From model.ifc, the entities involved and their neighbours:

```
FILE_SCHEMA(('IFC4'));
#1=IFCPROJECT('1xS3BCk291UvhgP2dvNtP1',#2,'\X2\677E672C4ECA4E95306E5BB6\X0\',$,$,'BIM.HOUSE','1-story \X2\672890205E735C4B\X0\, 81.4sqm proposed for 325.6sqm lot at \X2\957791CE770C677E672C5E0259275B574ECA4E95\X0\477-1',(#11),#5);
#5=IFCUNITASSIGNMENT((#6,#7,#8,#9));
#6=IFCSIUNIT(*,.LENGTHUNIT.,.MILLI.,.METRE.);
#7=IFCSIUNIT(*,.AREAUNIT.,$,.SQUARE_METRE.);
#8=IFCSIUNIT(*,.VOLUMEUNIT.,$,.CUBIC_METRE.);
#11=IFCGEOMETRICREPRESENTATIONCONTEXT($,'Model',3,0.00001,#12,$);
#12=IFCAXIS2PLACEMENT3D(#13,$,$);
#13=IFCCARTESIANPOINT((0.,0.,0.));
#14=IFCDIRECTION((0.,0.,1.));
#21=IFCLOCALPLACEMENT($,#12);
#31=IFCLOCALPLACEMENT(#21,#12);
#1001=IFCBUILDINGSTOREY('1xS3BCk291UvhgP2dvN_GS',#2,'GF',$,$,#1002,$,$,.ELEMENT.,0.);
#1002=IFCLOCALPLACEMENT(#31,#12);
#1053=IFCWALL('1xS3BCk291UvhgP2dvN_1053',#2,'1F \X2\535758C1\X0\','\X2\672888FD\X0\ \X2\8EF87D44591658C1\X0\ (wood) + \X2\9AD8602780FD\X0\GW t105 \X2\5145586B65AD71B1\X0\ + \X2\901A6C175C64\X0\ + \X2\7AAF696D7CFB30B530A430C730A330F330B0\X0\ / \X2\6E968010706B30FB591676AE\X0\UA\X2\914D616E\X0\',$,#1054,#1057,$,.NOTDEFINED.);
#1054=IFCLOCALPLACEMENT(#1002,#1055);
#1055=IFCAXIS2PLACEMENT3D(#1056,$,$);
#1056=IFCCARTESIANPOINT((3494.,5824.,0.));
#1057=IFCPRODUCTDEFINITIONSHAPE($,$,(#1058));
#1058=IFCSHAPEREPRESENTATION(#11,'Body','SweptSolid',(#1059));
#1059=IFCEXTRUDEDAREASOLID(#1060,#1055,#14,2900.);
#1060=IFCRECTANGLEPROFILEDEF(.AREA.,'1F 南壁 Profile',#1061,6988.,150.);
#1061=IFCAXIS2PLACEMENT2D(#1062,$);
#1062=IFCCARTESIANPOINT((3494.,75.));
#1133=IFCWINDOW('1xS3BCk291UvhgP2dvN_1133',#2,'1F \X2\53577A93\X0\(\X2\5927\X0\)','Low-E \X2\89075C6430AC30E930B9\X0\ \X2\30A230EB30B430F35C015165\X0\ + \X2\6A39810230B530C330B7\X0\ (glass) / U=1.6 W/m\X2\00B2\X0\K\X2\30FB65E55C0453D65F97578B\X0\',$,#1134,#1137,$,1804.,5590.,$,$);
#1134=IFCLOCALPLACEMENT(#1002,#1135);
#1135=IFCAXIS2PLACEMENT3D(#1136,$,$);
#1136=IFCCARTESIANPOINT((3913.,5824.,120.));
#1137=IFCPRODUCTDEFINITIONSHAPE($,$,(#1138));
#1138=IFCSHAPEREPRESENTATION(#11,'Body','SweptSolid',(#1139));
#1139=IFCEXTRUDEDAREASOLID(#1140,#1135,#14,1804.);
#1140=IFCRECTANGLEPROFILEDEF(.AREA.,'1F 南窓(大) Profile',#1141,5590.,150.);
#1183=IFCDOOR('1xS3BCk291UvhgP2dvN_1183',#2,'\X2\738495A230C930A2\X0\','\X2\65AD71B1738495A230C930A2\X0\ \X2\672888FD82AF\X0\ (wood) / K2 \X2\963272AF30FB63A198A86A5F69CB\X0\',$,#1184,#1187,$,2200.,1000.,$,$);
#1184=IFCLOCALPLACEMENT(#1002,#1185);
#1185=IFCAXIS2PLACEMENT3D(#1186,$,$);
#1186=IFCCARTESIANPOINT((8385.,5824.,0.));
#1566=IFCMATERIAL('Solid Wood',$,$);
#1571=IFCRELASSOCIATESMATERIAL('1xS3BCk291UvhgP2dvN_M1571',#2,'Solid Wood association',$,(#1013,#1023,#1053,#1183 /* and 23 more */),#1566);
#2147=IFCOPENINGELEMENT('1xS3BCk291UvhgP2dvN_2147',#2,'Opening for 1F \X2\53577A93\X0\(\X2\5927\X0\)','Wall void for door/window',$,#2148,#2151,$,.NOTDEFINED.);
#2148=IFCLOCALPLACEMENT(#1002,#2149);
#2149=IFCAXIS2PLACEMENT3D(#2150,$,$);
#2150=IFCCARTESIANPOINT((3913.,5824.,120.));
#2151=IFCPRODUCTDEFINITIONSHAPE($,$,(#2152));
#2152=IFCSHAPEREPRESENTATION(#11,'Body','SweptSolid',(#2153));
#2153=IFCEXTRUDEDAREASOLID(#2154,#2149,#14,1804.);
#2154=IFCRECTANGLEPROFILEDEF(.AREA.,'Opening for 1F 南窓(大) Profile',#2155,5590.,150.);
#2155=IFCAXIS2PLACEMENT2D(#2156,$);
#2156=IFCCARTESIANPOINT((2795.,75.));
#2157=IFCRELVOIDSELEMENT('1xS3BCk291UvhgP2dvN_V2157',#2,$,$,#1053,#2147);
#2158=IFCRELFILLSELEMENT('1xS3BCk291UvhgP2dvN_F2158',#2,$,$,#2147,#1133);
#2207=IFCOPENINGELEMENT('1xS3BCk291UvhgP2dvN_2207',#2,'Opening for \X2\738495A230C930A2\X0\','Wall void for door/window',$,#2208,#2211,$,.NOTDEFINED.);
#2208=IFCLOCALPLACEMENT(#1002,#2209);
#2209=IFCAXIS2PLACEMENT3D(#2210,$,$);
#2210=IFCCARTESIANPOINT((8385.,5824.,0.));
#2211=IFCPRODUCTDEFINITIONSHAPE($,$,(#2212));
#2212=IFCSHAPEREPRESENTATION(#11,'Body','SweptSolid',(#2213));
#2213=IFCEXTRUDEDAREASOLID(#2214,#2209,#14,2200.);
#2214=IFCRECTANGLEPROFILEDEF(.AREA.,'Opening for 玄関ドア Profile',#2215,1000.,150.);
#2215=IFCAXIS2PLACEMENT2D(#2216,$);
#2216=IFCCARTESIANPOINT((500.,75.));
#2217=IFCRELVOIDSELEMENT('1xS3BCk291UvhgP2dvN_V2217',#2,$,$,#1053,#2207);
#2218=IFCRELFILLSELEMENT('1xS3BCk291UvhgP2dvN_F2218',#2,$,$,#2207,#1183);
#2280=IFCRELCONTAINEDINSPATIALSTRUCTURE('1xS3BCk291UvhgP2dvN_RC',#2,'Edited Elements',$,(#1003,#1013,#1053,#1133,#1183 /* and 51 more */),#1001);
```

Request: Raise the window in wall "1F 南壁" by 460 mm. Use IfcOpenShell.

```python
import numpy as np
import ifcopenshell
import ifcopenshell.api.geometry
import ifcopenshell.util.placement
import ifcopenshell.util.unit

model = ifcopenshell.open("model.ifc")
unit_scale = ifcopenshell.util.unit.calculate_unit_scale(model)

window = model.by_id(1133)
opening = window.FillsVoids[0].RelatingOpeningElement
dz = 0.46 / unit_scale

shift = np.array([0.0, 0.0, dz])
# The window is not placed relative to its opening, so move both.
for product in (opening, window):
    matrix = ifcopenshell.util.placement.get_local_placement(product.ObjectPlacement)
    matrix[:3, 3] += shift
    ifcopenshell.api.geometry.edit_object_placement(model, product=product, matrix=matrix, is_si=False)

print(f"moved by {dz * unit_scale:+.3f} m")

model.write("model_edited.ifc")
```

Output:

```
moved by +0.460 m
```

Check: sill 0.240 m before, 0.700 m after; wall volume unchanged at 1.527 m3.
